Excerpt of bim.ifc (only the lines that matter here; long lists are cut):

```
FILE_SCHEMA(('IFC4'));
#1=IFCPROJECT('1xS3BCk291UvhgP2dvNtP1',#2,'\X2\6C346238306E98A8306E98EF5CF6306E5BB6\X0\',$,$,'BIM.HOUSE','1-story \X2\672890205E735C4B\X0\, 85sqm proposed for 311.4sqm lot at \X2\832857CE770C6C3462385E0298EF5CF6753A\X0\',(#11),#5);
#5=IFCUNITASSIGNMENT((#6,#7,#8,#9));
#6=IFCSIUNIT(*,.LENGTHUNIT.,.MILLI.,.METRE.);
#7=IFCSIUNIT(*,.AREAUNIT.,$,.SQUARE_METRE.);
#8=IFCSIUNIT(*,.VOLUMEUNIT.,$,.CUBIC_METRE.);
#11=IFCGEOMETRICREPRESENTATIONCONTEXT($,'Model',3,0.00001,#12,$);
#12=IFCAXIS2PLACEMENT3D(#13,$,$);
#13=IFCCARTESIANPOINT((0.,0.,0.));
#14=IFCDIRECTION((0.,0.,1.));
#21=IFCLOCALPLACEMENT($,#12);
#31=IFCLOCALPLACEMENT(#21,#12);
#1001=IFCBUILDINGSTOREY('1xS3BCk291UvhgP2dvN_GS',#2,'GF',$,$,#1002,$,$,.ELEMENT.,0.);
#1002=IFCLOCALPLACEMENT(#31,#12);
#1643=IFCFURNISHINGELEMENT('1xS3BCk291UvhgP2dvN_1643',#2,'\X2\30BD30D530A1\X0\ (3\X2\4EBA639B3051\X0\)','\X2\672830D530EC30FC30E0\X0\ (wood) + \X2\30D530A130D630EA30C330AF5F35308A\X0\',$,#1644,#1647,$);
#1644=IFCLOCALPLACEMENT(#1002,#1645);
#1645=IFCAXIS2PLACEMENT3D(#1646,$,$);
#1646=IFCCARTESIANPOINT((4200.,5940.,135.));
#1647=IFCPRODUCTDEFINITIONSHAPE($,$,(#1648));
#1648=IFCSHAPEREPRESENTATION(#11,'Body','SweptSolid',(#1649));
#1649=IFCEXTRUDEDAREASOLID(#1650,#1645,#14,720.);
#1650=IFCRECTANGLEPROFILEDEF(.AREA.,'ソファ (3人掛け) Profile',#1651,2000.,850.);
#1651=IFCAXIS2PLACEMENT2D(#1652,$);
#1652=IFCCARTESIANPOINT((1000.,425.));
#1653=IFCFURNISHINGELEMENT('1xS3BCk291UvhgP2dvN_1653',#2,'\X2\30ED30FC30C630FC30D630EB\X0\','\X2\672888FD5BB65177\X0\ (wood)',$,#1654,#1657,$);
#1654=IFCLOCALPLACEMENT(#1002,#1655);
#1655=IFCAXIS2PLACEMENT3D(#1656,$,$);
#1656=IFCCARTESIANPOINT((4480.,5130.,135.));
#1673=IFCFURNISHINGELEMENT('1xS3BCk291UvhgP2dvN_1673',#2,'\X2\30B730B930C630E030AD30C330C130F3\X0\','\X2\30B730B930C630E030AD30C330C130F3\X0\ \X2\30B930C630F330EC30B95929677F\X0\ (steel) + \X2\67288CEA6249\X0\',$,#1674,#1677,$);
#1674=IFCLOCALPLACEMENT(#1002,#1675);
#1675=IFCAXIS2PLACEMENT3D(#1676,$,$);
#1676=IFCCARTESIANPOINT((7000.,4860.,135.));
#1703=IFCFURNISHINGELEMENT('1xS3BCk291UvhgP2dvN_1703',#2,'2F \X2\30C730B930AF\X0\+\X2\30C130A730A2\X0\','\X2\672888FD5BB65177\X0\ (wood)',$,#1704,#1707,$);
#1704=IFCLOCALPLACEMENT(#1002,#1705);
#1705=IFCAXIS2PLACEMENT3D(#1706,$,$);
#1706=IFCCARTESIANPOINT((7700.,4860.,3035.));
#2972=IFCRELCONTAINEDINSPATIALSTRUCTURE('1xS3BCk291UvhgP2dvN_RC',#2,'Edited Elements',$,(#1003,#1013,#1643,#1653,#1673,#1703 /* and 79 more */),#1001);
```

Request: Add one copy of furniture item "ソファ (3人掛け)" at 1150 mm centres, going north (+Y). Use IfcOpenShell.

```python
import numpy as np
import ifcopenshell
import ifcopenshell.api.geometry
import ifcopenshell.api.root
import ifcopenshell.util.element
import ifcopenshell.util.placement
import ifcopenshell.util.unit

model = ifcopenshell.open("bim.ifc")
unit_scale = ifcopenshell.util.unit.calculate_unit_scale(model)


def reuse_history(source, copy):
    """copy_class also copies each property set's owner history, people and application; keep the originals."""
    for rel in copy.IsDefinedBy:
        if rel.is_a("IfcRelDefinesByProperties") and (history := rel.RelatingPropertyDefinition.OwnerHistory):
            rel.RelatingPropertyDefinition.OwnerHistory = source.OwnerHistory
            ifcopenshell.util.element.remove_deep2(model, history)


source = model.by_id(1643)
base = ifcopenshell.util.placement.get_local_placement(source.ObjectPlacement)
step = np.array([0.0, 1.0, 0.0]) * 1.15 / unit_scale

for i in range(1, 2):
    copy = ifcopenshell.api.root.copy_class(model, product=source)
    copy.Representation = ifcopenshell.util.element.copy_deep(
        model, source.Representation, exclude=["IfcGeometricRepresentationContext", "IfcRepresentationMap"]
    )
    reuse_history(source, copy)
    matrix = base.copy()
    matrix[:3, 3] += i * step
    print("added at", matrix[:3, 3].round(3) + 0.0)
    ifcopenshell.api.geometry.edit_object_placement(model, product=copy, matrix=matrix, is_si=False)

model.write("bim_edited.ifc")
```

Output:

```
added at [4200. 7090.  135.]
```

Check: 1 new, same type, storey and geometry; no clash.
